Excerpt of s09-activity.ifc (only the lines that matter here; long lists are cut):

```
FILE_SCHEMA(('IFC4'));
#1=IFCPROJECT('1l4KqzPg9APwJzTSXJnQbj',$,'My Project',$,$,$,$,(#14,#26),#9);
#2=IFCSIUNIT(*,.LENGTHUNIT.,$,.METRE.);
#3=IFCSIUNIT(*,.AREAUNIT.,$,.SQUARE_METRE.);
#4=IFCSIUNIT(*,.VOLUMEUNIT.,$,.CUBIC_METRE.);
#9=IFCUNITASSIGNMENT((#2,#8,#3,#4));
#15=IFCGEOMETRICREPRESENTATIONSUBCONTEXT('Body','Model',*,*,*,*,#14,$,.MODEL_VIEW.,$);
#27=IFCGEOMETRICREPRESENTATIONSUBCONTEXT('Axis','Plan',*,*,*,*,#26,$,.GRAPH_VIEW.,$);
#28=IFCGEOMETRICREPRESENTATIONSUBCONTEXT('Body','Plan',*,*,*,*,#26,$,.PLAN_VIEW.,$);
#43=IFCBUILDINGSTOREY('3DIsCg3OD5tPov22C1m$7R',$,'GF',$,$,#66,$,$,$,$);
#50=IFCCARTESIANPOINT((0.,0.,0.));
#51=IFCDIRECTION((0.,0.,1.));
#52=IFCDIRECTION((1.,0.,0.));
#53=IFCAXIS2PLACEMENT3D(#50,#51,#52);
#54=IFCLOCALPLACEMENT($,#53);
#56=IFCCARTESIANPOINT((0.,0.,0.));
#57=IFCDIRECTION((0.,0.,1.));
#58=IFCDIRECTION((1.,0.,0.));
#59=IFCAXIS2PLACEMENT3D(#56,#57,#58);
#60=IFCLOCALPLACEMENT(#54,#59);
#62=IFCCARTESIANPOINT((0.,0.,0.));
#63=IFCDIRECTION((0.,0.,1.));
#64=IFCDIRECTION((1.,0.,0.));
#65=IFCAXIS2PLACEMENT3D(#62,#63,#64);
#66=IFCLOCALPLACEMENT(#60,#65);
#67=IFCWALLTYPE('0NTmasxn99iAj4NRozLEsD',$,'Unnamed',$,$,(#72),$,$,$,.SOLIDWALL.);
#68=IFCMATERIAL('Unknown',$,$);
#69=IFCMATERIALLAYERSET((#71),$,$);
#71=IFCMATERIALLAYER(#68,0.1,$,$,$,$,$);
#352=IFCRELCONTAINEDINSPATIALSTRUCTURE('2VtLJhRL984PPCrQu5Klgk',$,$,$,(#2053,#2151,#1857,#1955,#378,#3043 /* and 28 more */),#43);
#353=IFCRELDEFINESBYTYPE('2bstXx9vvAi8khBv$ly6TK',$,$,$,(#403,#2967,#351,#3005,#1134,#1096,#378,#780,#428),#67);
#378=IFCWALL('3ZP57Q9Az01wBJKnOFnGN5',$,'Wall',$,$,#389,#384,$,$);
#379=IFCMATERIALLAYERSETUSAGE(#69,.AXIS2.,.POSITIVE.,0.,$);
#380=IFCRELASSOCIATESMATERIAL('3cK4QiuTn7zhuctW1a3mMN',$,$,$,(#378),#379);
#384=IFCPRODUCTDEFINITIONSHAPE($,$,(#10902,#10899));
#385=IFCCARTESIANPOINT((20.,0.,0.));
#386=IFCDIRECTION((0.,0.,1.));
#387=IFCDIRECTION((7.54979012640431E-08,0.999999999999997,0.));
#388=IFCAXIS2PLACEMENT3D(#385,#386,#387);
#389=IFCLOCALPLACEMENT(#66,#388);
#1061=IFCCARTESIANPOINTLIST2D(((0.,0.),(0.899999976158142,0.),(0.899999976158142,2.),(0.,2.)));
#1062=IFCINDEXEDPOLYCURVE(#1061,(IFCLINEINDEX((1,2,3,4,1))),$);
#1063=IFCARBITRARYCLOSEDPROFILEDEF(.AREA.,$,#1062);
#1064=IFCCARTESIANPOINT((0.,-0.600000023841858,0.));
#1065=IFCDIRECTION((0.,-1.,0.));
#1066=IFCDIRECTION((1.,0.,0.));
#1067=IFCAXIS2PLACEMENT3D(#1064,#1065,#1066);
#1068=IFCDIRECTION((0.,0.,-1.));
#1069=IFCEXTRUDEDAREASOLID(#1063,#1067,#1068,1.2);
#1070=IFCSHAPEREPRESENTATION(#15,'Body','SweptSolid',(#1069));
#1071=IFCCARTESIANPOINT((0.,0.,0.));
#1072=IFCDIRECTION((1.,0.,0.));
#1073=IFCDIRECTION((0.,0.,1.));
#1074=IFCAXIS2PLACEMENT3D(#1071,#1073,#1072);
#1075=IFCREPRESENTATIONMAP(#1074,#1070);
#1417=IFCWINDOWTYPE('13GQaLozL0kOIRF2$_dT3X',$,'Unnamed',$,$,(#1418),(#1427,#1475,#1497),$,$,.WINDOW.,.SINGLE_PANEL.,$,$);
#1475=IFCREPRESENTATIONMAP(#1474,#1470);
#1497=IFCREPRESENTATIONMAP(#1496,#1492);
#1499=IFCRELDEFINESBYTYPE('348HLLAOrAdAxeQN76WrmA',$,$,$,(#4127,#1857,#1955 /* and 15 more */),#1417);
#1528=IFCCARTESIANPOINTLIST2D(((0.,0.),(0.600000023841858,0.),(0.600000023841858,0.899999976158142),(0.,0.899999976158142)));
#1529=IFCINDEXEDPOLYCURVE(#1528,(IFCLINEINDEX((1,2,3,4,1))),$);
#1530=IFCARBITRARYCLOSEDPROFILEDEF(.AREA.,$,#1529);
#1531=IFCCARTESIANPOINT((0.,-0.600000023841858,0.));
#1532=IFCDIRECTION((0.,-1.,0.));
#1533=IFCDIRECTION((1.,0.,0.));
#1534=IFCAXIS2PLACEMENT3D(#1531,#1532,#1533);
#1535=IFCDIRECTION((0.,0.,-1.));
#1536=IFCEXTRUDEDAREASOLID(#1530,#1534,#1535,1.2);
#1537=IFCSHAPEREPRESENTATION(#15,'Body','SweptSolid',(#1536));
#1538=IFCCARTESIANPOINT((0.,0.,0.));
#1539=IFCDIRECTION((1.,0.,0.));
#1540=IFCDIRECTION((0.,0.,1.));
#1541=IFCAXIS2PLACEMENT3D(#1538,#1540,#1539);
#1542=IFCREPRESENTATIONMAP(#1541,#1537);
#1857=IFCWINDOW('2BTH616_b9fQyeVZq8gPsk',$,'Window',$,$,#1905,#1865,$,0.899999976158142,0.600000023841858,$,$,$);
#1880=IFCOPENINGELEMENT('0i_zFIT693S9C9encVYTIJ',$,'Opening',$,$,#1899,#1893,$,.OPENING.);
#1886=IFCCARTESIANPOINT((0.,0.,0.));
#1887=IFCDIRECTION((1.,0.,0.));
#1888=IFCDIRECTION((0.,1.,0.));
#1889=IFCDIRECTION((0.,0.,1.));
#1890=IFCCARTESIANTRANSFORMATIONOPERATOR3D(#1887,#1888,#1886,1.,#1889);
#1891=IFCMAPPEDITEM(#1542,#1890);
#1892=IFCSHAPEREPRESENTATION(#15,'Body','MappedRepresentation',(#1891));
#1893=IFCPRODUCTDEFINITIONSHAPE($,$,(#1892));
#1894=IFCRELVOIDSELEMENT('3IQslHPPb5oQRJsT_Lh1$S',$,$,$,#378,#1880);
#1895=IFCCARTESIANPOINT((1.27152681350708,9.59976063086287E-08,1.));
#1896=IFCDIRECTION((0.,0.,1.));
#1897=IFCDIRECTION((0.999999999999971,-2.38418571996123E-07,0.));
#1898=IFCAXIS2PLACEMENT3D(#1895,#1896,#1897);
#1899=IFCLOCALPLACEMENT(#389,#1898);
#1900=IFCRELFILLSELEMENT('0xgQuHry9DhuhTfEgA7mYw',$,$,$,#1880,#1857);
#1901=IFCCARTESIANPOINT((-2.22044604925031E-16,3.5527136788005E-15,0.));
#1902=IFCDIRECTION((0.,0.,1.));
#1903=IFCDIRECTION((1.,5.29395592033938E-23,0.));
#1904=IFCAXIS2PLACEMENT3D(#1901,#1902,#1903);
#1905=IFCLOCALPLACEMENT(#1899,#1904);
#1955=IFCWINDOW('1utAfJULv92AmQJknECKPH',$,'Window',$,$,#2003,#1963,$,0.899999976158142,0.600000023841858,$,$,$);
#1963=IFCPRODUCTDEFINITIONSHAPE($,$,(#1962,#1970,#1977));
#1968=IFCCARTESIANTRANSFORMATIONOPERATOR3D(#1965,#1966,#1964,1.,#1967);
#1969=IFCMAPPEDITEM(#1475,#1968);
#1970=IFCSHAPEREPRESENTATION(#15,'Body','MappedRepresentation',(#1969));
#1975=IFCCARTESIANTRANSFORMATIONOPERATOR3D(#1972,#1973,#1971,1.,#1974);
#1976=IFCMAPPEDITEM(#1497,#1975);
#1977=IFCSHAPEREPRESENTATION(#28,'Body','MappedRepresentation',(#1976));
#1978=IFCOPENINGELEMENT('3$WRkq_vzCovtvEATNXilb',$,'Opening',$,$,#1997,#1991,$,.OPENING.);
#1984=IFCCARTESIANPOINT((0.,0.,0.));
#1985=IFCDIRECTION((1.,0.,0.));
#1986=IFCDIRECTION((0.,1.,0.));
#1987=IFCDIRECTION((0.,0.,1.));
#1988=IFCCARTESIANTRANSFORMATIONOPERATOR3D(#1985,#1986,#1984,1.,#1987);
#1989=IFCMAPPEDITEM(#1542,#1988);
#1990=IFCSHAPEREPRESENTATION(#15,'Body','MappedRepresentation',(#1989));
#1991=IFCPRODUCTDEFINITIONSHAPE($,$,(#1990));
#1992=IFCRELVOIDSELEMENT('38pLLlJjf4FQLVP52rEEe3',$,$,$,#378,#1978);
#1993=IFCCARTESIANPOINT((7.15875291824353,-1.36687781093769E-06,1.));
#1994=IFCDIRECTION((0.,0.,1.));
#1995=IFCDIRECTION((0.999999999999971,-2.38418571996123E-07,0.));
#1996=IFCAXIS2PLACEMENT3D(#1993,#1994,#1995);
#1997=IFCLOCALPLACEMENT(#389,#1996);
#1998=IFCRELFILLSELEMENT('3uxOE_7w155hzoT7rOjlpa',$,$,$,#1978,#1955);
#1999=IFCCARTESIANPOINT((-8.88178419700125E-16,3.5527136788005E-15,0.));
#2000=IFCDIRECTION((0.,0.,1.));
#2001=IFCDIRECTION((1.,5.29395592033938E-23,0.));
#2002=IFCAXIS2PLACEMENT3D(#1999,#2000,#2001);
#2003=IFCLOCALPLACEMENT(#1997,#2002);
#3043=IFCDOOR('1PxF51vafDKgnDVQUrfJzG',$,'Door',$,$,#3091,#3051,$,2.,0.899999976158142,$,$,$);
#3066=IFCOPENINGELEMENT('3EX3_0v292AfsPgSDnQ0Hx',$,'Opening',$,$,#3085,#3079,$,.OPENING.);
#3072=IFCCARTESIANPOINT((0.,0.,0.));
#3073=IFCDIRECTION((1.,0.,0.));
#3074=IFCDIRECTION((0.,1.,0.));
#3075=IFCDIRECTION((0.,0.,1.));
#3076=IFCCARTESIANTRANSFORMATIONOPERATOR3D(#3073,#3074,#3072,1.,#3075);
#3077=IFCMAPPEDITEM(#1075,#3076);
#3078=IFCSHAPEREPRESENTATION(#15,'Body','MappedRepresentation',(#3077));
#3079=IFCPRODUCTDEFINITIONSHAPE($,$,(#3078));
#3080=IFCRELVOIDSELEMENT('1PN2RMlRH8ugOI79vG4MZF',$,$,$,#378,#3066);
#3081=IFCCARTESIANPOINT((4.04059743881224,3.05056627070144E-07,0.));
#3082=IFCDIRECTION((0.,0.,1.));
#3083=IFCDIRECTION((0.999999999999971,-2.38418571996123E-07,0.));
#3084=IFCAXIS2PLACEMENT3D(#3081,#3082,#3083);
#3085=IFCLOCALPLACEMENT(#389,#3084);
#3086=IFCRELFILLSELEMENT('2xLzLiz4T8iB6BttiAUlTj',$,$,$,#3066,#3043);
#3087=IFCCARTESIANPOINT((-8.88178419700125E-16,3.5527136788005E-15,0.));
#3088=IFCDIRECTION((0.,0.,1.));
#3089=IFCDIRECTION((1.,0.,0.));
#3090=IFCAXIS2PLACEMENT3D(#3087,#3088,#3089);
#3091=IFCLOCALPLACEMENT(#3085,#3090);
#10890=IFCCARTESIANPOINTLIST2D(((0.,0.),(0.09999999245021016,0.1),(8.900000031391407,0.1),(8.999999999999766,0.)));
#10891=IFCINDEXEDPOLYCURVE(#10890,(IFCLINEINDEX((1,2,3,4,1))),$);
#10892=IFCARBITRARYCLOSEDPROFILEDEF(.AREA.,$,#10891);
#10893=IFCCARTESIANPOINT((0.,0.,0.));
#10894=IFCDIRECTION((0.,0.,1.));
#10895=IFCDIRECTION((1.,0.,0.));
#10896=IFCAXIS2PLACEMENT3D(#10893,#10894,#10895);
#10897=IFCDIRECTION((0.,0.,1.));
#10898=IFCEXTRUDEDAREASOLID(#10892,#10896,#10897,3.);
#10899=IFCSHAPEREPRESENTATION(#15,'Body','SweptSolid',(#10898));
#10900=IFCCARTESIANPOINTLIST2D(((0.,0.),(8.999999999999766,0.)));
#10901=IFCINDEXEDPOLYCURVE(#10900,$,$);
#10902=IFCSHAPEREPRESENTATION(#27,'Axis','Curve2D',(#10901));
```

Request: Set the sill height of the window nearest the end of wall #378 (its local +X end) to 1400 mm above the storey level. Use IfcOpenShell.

```python
import numpy as np
import ifcopenshell
import ifcopenshell.api.geometry
import ifcopenshell.geom
import ifcopenshell.util.element
import ifcopenshell.util.placement
import ifcopenshell.util.shape
import ifcopenshell.util.unit

model = ifcopenshell.open("s09-activity.ifc")
unit_scale = ifcopenshell.util.unit.calculate_unit_scale(model)

window = model.by_guid("1utAfJULv92AmQJknECKPH")
opening = window.FillsVoids[0].RelatingOpeningElement
storey = ifcopenshell.util.element.get_container(window, ifc_class="IfcBuildingStorey")
level = ifcopenshell.util.placement.get_local_placement(storey.ObjectPlacement)[2, 3]

# The opening's origin need not be at the sill, so measure its lowest point.
shape = ifcopenshell.geom.create_shape(ifcopenshell.geom.settings(), opening)
bottom = ifcopenshell.util.shape.get_shape_bottom_elevation(shape, shape.geometry) / unit_scale
dz = level + 1.4 / unit_scale - bottom

shift = np.array([0.0, 0.0, dz])
# The window is placed relative to its opening, so it follows when the opening moves.
matrix = ifcopenshell.util.placement.get_local_placement(opening.ObjectPlacement)
matrix[:3, 3] += shift
ifcopenshell.api.geometry.edit_object_placement(
    model, product=opening, matrix=matrix, is_si=False, should_transform_children=True
)

print(f"moved by {dz * unit_scale:+.3f} m")

model.write("s09-activity_edited.ifc")
```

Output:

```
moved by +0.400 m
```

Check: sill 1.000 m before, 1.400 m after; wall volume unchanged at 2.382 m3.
